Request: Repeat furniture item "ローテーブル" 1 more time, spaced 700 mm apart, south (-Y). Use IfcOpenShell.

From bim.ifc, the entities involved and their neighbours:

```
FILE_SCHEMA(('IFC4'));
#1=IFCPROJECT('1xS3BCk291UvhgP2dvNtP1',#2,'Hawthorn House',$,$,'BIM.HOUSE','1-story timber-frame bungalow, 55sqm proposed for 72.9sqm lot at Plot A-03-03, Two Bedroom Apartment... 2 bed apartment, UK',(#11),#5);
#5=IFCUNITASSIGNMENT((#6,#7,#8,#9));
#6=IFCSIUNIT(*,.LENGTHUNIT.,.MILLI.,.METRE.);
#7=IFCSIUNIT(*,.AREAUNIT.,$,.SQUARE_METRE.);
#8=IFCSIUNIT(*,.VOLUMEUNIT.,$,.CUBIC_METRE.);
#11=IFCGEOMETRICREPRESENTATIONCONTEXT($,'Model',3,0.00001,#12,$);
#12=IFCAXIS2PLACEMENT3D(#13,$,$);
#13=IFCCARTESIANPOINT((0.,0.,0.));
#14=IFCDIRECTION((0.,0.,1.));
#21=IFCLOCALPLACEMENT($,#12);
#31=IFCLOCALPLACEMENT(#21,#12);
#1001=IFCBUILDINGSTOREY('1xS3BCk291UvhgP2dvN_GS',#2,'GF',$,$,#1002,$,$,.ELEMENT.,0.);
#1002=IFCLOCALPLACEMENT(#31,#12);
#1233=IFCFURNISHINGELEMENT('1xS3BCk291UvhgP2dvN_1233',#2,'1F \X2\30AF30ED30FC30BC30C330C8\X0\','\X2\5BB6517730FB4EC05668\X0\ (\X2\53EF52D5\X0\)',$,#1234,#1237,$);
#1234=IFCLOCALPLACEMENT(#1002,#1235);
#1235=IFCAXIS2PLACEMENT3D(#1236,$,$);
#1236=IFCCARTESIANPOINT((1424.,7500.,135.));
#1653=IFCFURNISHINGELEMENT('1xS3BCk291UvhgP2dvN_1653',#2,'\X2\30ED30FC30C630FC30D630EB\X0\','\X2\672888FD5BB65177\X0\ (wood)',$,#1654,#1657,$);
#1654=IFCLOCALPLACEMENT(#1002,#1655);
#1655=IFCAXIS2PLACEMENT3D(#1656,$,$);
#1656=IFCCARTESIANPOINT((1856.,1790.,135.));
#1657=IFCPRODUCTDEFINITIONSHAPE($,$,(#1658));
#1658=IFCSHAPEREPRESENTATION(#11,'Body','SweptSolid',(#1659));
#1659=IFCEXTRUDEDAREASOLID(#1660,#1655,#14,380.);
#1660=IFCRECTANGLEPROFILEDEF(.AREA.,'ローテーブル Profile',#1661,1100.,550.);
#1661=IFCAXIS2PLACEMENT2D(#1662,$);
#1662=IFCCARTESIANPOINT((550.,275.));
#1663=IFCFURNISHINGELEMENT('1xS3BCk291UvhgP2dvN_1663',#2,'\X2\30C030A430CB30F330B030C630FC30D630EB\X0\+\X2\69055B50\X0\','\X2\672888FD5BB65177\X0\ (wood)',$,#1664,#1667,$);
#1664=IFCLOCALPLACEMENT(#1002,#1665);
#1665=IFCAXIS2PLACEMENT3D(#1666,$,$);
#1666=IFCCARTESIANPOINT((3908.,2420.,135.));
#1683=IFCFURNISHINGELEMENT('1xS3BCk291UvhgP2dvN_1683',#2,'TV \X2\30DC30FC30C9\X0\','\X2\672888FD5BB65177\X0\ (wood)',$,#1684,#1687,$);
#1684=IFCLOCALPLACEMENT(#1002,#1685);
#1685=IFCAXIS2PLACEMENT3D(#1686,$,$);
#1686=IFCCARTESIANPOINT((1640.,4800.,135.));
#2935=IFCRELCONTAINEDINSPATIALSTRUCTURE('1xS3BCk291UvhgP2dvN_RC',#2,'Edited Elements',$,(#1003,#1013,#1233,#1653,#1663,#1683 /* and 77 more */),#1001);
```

```python
import numpy as np
import ifcopenshell
import ifcopenshell.api.geometry
import ifcopenshell.api.root
import ifcopenshell.util.element
import ifcopenshell.util.placement

model = ifcopenshell.open("bim.ifc")


def reuse_history(source, copy):
    """copy_class also copies each property set's owner history, people and application; keep the originals."""
    for rel in copy.IsDefinedBy:
        if rel.is_a("IfcRelDefinesByProperties") and (history := rel.RelatingPropertyDefinition.OwnerHistory):
            rel.RelatingPropertyDefinition.OwnerHistory = source.OwnerHistory
            ifcopenshell.util.element.remove_deep2(model, history)


source = model.by_id(1653)
base = ifcopenshell.util.placement.get_local_placement(source.ObjectPlacement)
step = np.array([0.0, -1.0, 0.0]) * 700.0

for i in range(1, 2):
    copy = ifcopenshell.api.root.copy_class(model, product=source)
    copy.Representation = ifcopenshell.util.element.copy_deep(
        model, source.Representation, exclude=["IfcGeometricRepresentationContext", "IfcRepresentationMap"]
    )
    reuse_history(source, copy)
    matrix = base.copy()
    matrix[:3, 3] += i * step
    print("added at", matrix[:3, 3].round(3) + 0.0)
    ifcopenshell.api.geometry.edit_object_placement(model, product=copy, matrix=matrix, is_si=False)

model.write("bim_v2.ifc")
```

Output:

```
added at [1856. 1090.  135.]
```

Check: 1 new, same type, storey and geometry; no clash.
